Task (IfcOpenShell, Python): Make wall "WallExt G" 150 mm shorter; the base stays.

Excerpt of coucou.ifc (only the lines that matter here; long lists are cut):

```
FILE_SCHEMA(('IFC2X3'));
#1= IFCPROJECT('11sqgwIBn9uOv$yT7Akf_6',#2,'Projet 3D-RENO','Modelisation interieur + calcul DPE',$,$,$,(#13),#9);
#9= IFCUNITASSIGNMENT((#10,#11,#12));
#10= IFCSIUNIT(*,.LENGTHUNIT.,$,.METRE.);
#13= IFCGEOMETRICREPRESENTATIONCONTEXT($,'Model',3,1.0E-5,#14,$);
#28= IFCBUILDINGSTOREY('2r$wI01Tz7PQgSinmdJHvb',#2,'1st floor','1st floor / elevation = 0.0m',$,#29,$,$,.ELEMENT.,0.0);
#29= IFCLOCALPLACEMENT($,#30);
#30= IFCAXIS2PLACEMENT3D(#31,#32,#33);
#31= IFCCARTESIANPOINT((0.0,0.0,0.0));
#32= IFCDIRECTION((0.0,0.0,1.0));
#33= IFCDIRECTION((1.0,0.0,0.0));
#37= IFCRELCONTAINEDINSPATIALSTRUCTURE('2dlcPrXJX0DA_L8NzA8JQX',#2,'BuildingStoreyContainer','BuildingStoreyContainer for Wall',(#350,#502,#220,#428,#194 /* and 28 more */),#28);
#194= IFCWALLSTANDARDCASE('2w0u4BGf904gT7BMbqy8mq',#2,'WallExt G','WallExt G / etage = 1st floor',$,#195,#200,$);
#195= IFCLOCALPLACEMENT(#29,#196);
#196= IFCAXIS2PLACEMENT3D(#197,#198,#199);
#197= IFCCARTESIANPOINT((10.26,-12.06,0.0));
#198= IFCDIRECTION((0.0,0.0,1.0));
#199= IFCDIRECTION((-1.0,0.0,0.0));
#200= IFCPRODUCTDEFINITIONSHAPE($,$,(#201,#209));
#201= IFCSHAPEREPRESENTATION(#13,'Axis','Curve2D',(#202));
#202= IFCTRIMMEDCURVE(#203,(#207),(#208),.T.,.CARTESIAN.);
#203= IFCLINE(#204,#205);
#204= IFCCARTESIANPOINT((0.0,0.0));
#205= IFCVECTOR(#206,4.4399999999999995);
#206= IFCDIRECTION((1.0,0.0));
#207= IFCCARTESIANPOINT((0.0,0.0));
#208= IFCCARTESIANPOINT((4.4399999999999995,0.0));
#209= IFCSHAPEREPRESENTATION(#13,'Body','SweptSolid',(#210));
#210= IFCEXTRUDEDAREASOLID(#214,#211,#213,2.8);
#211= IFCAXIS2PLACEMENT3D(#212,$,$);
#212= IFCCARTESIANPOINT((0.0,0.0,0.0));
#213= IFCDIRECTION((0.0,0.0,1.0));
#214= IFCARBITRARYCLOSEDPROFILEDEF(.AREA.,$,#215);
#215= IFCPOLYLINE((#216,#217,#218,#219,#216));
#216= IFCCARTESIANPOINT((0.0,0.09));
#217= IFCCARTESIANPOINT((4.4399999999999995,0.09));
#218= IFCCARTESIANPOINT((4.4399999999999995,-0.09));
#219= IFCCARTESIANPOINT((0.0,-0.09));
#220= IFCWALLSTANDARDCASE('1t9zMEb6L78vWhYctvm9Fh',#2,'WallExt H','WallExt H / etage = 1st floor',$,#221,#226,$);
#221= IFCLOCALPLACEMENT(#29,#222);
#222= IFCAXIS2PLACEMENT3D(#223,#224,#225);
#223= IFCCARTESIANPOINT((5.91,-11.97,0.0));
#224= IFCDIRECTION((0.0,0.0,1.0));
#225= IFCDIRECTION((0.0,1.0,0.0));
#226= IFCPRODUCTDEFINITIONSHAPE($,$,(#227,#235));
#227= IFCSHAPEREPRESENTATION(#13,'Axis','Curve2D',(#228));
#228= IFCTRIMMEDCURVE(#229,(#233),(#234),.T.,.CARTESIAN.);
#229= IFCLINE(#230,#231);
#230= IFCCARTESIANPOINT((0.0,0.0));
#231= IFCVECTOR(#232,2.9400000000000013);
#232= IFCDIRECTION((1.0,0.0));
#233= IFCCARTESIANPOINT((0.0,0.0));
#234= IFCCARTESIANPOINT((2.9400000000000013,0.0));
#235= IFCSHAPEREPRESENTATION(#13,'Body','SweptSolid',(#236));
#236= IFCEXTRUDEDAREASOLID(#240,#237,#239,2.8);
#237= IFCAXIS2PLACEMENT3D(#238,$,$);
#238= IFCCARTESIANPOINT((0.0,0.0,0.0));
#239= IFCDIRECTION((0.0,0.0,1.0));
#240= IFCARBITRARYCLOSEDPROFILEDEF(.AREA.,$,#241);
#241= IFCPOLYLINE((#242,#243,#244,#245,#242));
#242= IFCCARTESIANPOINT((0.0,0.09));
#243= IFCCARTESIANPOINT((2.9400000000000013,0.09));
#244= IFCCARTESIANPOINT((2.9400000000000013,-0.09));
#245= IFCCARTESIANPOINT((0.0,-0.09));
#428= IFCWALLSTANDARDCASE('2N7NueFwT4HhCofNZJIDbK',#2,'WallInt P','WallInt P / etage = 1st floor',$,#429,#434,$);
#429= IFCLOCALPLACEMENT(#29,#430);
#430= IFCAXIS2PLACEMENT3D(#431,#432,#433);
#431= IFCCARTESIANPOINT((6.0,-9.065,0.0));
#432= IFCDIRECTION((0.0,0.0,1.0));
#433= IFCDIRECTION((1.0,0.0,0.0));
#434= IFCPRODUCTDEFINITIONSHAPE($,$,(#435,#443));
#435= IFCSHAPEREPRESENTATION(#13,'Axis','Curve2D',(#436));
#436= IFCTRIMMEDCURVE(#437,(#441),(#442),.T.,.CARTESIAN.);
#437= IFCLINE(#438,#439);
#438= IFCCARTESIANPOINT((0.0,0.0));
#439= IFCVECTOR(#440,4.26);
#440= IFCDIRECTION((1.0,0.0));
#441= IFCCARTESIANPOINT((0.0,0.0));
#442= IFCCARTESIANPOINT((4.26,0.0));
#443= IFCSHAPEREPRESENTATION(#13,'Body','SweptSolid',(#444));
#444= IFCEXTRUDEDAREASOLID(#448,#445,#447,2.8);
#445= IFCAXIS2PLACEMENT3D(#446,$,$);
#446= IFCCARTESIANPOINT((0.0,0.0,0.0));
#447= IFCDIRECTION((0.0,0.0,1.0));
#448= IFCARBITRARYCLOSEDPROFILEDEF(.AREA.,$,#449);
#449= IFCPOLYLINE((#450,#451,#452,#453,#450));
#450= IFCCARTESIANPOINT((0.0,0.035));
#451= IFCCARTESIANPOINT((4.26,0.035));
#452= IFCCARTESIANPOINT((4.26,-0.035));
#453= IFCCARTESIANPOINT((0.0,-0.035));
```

```python
import ifcopenshell
import ifcopenshell.geom
import ifcopenshell.util.shape
import ifcopenshell.util.unit

model = ifcopenshell.open("coucou.ifc")
unit_scale = ifcopenshell.util.unit.calculate_unit_scale(model)
settings = ifcopenshell.geom.settings()


def volume(element):
    """Net volume in cubic metres, openings subtracted."""
    shape = ifcopenshell.geom.create_shape(settings, element)
    return ifcopenshell.util.shape.get_volume(shape.geometry)


wall = model.by_guid("2w0u4BGf904gT7BMbqy8mq")
before = volume(wall)

body = next(r for r in wall.Representation.Representations if r.RepresentationIdentifier == "Body")
solid = body.Items[0]
old_height = solid.Depth
solid.Depth -= 0.15 / unit_scale
after = volume(wall)

print(f"height {old_height:g} -> {solid.Depth:g}, volume {before:.3f} -> {after:.3f} m3")

model.write("coucou_updated.ifc")
```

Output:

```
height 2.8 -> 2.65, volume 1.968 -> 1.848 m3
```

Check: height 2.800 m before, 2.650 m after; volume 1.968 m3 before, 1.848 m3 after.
